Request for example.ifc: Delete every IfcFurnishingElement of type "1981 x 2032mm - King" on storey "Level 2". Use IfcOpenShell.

First a look at what the model holds.

```python
import ifcopenshell
import ifcopenshell.util.element

model = ifcopenshell.open("example.ifc")
print(model.schema)
storey = next(s for s in model.by_type("IfcBuildingStorey") if s.Name == "Level 2")
furniture = [e for e in ifcopenshell.util.element.get_decomposition(storey) if e.is_a("IfcFurnishingElement")]
seen = {}
for e in furniture:
    element_type = ifcopenshell.util.element.get_type(e)
    name = element_type.Name if element_type not in (None, e) else None
    seen[name] = seen.get(name, 0) + 1
for name, count in sorted(seen.items(), key=str):
    print(count, "x", name)
```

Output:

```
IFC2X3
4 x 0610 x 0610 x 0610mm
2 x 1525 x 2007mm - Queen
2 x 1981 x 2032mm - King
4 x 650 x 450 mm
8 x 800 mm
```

```python
import ifcopenshell
import ifcopenshell.api.root
import ifcopenshell.util.element

model = ifcopenshell.open("example.ifc")

storey = next(s for s in model.by_type("IfcBuildingStorey") if s.Name == "Level 2")
furniture = [e for e in ifcopenshell.util.element.get_decomposition(storey) if e.is_a("IfcFurnishingElement")]
targets = [e for e in furniture if (t := ifcopenshell.util.element.get_type(e)) not in (None, e) and t.Name == "1981 x 2032mm - King"]

for e in targets:
    ifcopenshell.api.root.remove_product(model, product=e)
print(len(targets), "removed")

model.write("example_rev.ifc")
```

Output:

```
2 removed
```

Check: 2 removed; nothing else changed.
